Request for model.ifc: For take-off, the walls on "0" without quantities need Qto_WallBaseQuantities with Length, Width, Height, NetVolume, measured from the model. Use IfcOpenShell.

First a look at what the model holds.

```python
import ifcopenshell
import ifcopenshell.util.element
import ifcopenshell.util.unit

model = ifcopenshell.open("model.ifc")
print(model.schema)
for unit_type in ("LENGTHUNIT", "AREAUNIT", "VOLUMEUNIT"):
    print(unit_type, ifcopenshell.util.unit.calculate_unit_scale(model, unit_type))
storey = next(s for s in model.by_type("IfcBuildingStorey") if s.Name == "0")
walls = [e for e in ifcopenshell.util.element.get_decomposition(storey) if e.is_a("IfcWall")]
for e in sorted(walls, key=lambda e: e.id()):
    print(e.id(), e.is_a(), e.Name, list(ifcopenshell.util.element.get_psets(e, qtos_only=True)), sep=" | ")
```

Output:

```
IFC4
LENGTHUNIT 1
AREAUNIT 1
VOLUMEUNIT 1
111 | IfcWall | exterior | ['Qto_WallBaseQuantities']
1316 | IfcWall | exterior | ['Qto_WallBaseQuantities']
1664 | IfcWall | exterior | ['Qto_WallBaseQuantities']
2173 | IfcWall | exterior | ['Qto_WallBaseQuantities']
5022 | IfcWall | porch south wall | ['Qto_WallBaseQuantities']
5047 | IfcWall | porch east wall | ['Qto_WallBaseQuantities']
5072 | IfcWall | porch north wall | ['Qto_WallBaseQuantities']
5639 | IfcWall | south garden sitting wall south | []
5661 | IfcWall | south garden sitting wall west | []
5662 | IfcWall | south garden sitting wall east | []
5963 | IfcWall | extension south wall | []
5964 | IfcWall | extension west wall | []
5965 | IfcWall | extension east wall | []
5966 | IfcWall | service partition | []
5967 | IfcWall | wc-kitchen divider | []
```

```python
import ifcopenshell
import ifcopenshell.api.pset
import ifcopenshell.geom
import ifcopenshell.util.element
import ifcopenshell.util.shape
import ifcopenshell.util.unit

model = ifcopenshell.open("model.ifc")
unit_scale = ifcopenshell.util.unit.calculate_unit_scale(model)
volume_scale = ifcopenshell.util.unit.calculate_unit_scale(model, "VOLUMEUNIT")
settings = ifcopenshell.geom.settings()

storey = next(s for s in model.by_type("IfcBuildingStorey") if s.Name == "0")
walls = [e for e in ifcopenshell.util.element.get_decomposition(storey) if e.is_a("IfcWall")]

for e in sorted(walls, key=lambda e: e.id()):
    if ifcopenshell.util.element.get_psets(e, qtos_only=True, should_inherit=False):
        continue
    # Geometry comes back in metres, in the element's own axes.
    shape = ifcopenshell.geom.create_shape(settings, e)
    values = {
        "Length": ifcopenshell.util.shape.get_x(shape.geometry) / unit_scale,
        "Width": ifcopenshell.util.shape.get_y(shape.geometry) / unit_scale,
        "Height": ifcopenshell.util.shape.get_z(shape.geometry) / unit_scale,
        "NetVolume": ifcopenshell.util.shape.get_volume(shape.geometry) / volume_scale,
    }
    qto = ifcopenshell.api.pset.add_qto(model, product=e, name="Qto_WallBaseQuantities")
    ifcopenshell.api.pset.edit_qto(model, qto=qto, properties=values)
    print(e.id(), {k: round(v, 3) for k, v in values.items()})

model.write("model_updated.ifc")
```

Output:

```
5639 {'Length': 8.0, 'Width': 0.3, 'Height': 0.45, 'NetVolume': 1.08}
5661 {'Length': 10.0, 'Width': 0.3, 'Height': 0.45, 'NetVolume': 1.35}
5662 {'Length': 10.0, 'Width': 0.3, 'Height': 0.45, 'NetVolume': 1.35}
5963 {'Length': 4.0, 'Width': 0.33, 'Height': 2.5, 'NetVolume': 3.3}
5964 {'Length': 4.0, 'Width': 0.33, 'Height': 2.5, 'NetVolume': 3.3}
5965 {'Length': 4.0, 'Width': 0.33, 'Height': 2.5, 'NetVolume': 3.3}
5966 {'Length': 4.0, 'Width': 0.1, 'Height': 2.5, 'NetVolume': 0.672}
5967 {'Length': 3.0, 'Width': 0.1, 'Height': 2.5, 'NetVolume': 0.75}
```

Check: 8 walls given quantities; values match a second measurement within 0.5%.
